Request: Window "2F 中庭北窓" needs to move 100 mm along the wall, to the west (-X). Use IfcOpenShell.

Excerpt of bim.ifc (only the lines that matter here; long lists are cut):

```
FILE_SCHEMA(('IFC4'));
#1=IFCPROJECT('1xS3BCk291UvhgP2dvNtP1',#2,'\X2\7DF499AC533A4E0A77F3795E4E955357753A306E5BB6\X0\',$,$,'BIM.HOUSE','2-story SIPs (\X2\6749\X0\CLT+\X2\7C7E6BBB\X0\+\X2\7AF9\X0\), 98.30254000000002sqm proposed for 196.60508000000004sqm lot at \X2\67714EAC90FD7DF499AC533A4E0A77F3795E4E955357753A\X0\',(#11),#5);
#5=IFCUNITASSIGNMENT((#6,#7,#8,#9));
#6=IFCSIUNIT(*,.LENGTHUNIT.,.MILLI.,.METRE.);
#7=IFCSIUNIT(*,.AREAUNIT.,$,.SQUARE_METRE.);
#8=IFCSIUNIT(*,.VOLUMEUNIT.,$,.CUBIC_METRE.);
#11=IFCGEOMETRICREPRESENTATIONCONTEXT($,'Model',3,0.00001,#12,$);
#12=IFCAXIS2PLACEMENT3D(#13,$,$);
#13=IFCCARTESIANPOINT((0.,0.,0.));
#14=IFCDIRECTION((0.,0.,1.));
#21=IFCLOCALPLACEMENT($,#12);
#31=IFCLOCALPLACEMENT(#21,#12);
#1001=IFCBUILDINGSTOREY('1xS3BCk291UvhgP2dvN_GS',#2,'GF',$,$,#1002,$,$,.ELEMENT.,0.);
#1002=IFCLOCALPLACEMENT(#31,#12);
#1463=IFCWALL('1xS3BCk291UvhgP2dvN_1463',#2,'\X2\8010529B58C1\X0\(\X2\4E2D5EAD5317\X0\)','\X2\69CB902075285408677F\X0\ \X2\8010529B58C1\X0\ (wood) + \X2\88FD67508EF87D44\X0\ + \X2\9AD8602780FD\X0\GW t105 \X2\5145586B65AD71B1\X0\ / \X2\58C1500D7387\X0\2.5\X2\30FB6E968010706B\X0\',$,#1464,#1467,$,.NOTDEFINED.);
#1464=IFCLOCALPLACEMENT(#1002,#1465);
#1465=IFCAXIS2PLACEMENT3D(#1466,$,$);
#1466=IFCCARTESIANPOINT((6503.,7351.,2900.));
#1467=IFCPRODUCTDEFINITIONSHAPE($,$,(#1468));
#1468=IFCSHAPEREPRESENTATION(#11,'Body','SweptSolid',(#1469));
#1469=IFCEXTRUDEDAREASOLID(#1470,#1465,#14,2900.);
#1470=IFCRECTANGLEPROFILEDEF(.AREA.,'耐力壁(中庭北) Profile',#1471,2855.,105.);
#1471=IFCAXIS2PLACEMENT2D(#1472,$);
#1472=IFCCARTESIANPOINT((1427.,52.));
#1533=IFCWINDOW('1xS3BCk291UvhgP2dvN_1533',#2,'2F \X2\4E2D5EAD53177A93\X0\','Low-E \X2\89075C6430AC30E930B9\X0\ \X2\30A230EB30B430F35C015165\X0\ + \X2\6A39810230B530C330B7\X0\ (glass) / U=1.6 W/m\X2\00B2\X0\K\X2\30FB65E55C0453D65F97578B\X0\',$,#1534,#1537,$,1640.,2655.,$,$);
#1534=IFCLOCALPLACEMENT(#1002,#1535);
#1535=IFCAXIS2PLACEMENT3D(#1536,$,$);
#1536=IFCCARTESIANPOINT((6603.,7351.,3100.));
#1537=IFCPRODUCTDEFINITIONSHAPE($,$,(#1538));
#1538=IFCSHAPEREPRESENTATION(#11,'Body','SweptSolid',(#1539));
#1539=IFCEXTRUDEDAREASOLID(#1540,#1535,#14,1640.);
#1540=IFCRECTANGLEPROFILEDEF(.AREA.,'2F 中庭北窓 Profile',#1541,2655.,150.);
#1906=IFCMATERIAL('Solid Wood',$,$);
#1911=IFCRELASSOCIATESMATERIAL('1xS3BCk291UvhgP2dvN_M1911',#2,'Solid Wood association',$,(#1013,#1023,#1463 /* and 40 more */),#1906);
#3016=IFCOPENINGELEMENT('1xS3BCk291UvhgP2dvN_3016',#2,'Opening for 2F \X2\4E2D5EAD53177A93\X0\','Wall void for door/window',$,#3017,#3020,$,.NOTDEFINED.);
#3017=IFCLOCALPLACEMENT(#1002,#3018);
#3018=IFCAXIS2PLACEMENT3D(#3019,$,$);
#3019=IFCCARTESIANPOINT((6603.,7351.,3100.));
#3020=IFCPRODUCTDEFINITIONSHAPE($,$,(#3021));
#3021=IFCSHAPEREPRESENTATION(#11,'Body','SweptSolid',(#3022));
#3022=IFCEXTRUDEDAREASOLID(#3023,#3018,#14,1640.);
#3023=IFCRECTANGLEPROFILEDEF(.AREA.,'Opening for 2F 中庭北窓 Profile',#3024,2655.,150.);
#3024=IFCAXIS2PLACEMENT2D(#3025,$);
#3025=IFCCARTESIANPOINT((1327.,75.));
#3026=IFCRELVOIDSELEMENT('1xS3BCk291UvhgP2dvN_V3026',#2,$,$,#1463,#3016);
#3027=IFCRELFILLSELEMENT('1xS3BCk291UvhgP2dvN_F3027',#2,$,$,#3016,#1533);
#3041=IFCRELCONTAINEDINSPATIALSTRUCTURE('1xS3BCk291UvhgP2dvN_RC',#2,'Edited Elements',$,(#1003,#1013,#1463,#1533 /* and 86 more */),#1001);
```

```python
import ifcopenshell
import ifcopenshell.api.geometry
import ifcopenshell.util.placement

model = ifcopenshell.open("bim.ifc")

window = model.by_id(1533)
opening = window.FillsVoids[0].RelatingOpeningElement
wall = opening.VoidsElements[0].RelatingBuildingElement

wall_matrix = ifcopenshell.util.placement.get_local_placement(wall.ObjectPlacement)
shift = wall_matrix[:3, 0] * -100.0
before = ifcopenshell.util.placement.get_local_placement(window.ObjectPlacement)[:3, 3].copy()

# The window is not placed relative to its opening, so move both.
for product in (opening, window):
    matrix = ifcopenshell.util.placement.get_local_placement(product.ObjectPlacement)
    matrix[:3, 3] += shift
    ifcopenshell.api.geometry.edit_object_placement(model, product=product, matrix=matrix, is_si=False)

after = ifcopenshell.util.placement.get_local_placement(window.ObjectPlacement)[:3, 3]
print("window moved by", (after - before).round(3) + 0.0)

model.write("bim_v2.ifc")
```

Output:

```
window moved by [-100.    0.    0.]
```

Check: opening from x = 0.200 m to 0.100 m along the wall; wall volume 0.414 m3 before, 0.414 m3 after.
